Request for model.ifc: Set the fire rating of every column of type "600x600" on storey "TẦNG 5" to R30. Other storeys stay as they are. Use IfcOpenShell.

First a look at what the model holds.

```python
import ifcopenshell
import ifcopenshell.util.element

model = ifcopenshell.open("model.ifc")
print(model.schema)
storey = next(s for s in model.by_type("IfcBuildingStorey") if s.Name == "TẦNG 5")
columns = [e for e in ifcopenshell.util.element.get_decomposition(storey) if e.is_a("IfcColumn")]
seen = {}
for e in columns:
    element_type = ifcopenshell.util.element.get_type(e)
    key = (element_type.Name if element_type != e and element_type else None, ifcopenshell.util.element.get_pset(e, "Pset_ColumnCommon", "FireRating"))
    seen[key] = seen.get(key, 0) + 1
for (name, value), count in sorted(seen.items(), key=str):
    print(count, "x", name, "|", value)
```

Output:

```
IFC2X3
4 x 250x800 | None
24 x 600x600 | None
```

```python
import ifcopenshell
import ifcopenshell.api.pset
import ifcopenshell.util.element

model = ifcopenshell.open("model.ifc")

storey = next(s for s in model.by_type("IfcBuildingStorey") if s.Name == "TẦNG 5")
columns = [e for e in ifcopenshell.util.element.get_decomposition(storey) if e.is_a("IfcColumn")]

count = 0
for e in columns:
    element_type = ifcopenshell.util.element.get_type(e)
    if element_type in (None, e) or element_type.Name != "600x600":
        continue
    # add_pset returns the element's existing set when there is one.
    pset = ifcopenshell.api.pset.add_pset(model, product=e, name="Pset_ColumnCommon")
    ifcopenshell.api.pset.edit_pset(model, pset=pset, properties={"FireRating": "R30"})
    count += 1

print(count, "columns updated")

model.write("model_rev.ifc")
```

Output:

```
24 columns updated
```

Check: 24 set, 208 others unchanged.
